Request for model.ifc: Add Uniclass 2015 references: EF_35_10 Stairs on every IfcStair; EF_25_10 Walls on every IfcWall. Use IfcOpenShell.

First a look at what the model holds.

```python
import ifcopenshell

model = ifcopenshell.open("model.ifc")
print(model.schema)
print("classifications:", [c.Name for c in model.by_type("IfcClassification")])
for ifc_class in ("IfcDoor", "IfcRoof", "IfcStair", "IfcWall", "IfcWindow"):
    print(ifc_class, len(model.by_type(ifc_class)))
```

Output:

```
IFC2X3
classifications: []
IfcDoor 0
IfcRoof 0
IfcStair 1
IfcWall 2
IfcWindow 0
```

```python
import ifcopenshell
import ifcopenshell.api.classification

model = ifcopenshell.open("model.ifc")

# IFC2X3 requires Source and Edition and has no link from the project to the system.
system = model.create_entity("IfcClassification", Source="NBS", Edition="2015", Name="Uniclass 2015")

codes = {
    "IfcStair": ("EF_35_10", "Stairs"),
    "IfcWall": ("EF_25_10", "Walls"),
}
for ifc_class, (code, name) in codes.items():
    products = model.by_type(ifc_class)
    ifcopenshell.api.classification.add_reference(
        model, products=products, classification=system, identification=code, name=name
    )
    print(code, len(products))

model.write("model_updated.ifc")
```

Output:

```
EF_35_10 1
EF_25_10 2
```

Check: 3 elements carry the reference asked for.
